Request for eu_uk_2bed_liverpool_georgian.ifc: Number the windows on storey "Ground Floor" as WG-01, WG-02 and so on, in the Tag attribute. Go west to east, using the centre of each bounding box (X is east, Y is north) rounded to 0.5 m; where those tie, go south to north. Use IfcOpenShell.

First a look at what the model holds.

```python
import ifcopenshell
import ifcopenshell.util.element
import ifcopenshell.util.placement

model = ifcopenshell.open("eu_uk_2bed_liverpool_georgian.ifc")
print(model.schema)
storey = next(s for s in model.by_type("IfcBuildingStorey") if s.Name == "Ground Floor")
windows = [e for e in ifcopenshell.util.element.get_decomposition(storey) if e.is_a("IfcWindow")]
for e in sorted(windows, key=lambda e: e.id()):
    origin = ifcopenshell.util.placement.get_local_placement(e.ObjectPlacement)[:3, 3]
    print(e.id(), e.Tag, e.Name, origin.round(2) + 0.0, sep=" | ")
```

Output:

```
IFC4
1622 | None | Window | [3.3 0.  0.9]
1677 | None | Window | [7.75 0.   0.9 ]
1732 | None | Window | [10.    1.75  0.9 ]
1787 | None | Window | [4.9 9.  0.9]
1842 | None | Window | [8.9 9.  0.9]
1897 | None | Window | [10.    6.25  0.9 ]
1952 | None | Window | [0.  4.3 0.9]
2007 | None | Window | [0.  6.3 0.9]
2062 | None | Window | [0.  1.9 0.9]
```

```python
import ifcopenshell
import ifcopenshell.geom
import ifcopenshell.util.element
import ifcopenshell.util.shape

model = ifcopenshell.open("eu_uk_2bed_liverpool_georgian.ifc")
settings = ifcopenshell.geom.settings()
settings.set("use-world-coords", True)


def centre(element):
    shape = ifcopenshell.geom.create_shape(settings, element)
    return ifcopenshell.util.shape.get_bbox_centroid(shape.geometry)


storey = next(s for s in model.by_type("IfcBuildingStorey") if s.Name == "Ground Floor")
windows = [e for e in ifcopenshell.util.element.get_decomposition(storey) if e.is_a("IfcWindow")]

# Insertion points can sit at a corner or the storey origin, so sort by the geometry (in metres).
centres = {e: centre(e) for e in windows}
windows.sort(key=lambda e: (round(centres[e][0] / 0.5), centres[e][1]))

for i, e in enumerate(windows, start=1):
    number = f"WG-{i:02d}"
    e.Tag = number
    print(e.id(), number)

model.write("eu_uk_2bed_liverpool_georgian_v2.ifc")
```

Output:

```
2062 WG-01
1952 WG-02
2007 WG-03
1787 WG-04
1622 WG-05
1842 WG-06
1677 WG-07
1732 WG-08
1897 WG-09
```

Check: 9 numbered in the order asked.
